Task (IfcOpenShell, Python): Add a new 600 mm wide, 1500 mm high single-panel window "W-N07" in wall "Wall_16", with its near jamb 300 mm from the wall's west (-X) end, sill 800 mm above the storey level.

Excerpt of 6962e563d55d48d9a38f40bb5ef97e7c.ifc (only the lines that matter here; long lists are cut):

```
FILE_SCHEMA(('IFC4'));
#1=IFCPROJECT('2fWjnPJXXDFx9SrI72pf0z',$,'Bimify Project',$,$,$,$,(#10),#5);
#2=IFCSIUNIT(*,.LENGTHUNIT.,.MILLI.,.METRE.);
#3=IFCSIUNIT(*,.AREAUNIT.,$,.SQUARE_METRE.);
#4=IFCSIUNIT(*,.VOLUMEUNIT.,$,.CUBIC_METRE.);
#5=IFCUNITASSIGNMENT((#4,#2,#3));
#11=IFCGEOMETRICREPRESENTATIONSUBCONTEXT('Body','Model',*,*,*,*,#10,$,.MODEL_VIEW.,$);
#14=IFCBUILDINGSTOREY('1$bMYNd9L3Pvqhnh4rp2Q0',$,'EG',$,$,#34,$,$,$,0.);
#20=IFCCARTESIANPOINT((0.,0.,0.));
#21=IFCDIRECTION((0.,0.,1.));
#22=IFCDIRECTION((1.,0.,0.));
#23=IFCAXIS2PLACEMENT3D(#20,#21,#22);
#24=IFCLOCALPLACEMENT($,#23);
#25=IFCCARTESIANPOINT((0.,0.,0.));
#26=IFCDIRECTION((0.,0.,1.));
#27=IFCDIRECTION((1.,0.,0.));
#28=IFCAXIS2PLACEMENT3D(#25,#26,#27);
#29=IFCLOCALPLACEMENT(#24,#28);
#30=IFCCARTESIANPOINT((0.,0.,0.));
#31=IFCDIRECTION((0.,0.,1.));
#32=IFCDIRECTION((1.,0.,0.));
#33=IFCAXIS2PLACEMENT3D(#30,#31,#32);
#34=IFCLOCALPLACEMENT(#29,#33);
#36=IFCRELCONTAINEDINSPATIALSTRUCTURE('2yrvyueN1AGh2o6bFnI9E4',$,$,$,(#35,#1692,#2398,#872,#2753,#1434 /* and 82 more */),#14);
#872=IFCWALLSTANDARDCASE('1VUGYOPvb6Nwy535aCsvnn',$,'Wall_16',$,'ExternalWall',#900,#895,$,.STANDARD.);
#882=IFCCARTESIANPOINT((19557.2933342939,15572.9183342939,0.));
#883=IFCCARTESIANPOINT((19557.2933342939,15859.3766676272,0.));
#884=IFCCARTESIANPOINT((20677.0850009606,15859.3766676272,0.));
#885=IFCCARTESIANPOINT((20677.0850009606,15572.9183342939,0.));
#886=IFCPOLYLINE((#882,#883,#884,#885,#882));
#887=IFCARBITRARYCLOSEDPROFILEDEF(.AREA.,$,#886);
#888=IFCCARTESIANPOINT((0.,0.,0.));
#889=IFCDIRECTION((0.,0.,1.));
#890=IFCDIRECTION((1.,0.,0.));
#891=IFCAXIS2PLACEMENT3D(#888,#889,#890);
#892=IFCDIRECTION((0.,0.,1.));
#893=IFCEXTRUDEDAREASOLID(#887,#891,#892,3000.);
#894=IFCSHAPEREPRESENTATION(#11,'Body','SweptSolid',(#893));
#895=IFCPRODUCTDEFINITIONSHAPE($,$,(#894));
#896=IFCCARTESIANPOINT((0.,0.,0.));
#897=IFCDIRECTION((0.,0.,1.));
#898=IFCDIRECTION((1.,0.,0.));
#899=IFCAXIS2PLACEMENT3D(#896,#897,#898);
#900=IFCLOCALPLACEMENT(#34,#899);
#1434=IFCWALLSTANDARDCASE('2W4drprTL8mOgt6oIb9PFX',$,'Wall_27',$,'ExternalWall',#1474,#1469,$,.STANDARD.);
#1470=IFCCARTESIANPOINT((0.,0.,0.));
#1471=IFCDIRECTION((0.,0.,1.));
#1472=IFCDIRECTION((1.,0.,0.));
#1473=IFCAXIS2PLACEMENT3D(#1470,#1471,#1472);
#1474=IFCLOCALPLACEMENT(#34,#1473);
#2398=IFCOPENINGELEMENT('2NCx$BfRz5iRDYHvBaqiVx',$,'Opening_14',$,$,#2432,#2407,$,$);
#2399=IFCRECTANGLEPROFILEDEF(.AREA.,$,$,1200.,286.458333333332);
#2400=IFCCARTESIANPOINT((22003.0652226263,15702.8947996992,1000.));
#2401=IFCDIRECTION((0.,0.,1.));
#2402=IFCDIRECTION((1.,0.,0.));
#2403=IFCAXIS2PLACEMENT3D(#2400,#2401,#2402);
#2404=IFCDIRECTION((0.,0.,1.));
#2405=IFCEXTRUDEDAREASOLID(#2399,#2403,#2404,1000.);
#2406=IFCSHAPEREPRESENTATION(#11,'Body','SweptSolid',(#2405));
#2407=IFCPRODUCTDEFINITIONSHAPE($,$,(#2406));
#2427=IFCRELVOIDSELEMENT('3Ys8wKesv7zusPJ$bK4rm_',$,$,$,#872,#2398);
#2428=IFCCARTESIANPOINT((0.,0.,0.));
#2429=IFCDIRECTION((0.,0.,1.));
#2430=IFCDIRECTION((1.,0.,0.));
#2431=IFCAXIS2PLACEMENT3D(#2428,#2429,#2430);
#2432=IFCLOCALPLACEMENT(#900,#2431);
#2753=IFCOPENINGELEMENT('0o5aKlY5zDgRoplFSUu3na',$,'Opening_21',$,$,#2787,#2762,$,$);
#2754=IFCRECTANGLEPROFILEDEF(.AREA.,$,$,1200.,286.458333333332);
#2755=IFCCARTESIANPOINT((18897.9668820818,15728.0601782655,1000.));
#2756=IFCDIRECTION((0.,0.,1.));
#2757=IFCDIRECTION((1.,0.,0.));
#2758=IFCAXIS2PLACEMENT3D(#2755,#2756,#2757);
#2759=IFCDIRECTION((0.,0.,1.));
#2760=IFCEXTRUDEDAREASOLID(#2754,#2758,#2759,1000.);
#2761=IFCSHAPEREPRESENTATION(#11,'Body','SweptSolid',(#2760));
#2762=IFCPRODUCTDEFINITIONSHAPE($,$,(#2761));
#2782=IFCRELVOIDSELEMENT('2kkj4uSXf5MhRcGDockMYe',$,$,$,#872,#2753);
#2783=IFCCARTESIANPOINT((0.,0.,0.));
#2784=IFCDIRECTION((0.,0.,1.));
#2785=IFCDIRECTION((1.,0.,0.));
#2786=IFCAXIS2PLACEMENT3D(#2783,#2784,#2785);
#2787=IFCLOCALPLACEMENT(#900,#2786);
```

```python
import numpy as np
import ifcopenshell
import ifcopenshell.api.feature
import ifcopenshell.api.geometry
import ifcopenshell.api.root
import ifcopenshell.api.spatial
import ifcopenshell.geom
import ifcopenshell.util.element
import ifcopenshell.util.placement
import ifcopenshell.util.representation
import ifcopenshell.util.shape
import ifcopenshell.util.unit

model = ifcopenshell.open("6962e563d55d48d9a38f40bb5ef97e7c.ifc")
unit_scale = ifcopenshell.util.unit.calculate_unit_scale(model)
settings = ifcopenshell.geom.settings()


def volume(element):
    """Net volume in cubic metres, openings subtracted."""
    shape = ifcopenshell.geom.create_shape(settings, element)
    return ifcopenshell.util.shape.get_volume(shape.geometry)


wall = model.by_guid("1VUGYOPvb6Nwy535aCsvnn")
storey = ifcopenshell.util.element.get_container(wall, ifc_class="IfcBuildingStorey")
context = ifcopenshell.util.representation.get_context(model, "Model", "Body", "MODEL_VIEW")
before = volume(wall)

width, height, from_end, sill = 0.6, 1.5, 0.3, 0.8  # metres

# The wall runs along its own X axis, and the end named is its -X end.
wall_shape = ifcopenshell.geom.create_shape(settings, wall)
x, y, z = ifcopenshell.util.shape.get_vertices(wall_shape.geometry).T
start = x.min() + from_end
face, thickness = float(y.min()), float(y.max() - y.min())
wall_matrix = ifcopenshell.util.placement.get_local_placement(wall.ObjectPlacement)
level = ifcopenshell.util.placement.get_local_placement(storey.ObjectPlacement)[2, 3]


def in_wall(x, y):
    """Placement at x, y metres in the wall's axes, at sill height."""
    matrix = wall_matrix.copy()
    matrix[:, 3] = wall_matrix @ np.array([x / unit_scale, y / unit_scale, 0.0, 1.0])
    matrix[2, 3] = level + sill / unit_scale
    return matrix


# Opening: a box that overshoots both wall faces by 50 mm.
opening = ifcopenshell.api.root.create_entity(model, ifc_class="IfcOpeningElement", predefined_type="OPENING")
box = ifcopenshell.api.geometry.add_wall_representation(
    model, context=context, length=width, height=height, thickness=thickness + 0.1
)
ifcopenshell.api.geometry.assign_representation(model, product=opening, representation=box)
ifcopenshell.api.geometry.edit_object_placement(model, product=opening, matrix=in_wall(start, face - 0.05), is_si=False)
ifcopenshell.api.feature.add_feature(model, feature=opening, element=wall)

window = ifcopenshell.api.root.create_entity(model, ifc_class="IfcWindow", name="W-N07", predefined_type="WINDOW")
window.OverallWidth, window.OverallHeight = width / unit_scale, height / unit_scale
window.PartitioningType = "SINGLE_PANEL"
body = ifcopenshell.api.geometry.add_window_representation(
    model,
    context=context,
    overall_width=window.OverallWidth,
    overall_height=window.OverallHeight,
    partition_type="SINGLE_PANEL",
)
ifcopenshell.api.geometry.assign_representation(model, product=window, representation=body)
ifcopenshell.api.spatial.assign_container(model, products=[window], relating_structure=storey)
ifcopenshell.api.feature.add_filling(model, opening=opening, element=window)

# Centre the window in the wall's thickness.
ifcopenshell.api.geometry.edit_object_placement(model, product=window, matrix=in_wall(start, face), is_si=False)
window_shape = ifcopenshell.geom.create_shape(settings, window)
depth = ifcopenshell.util.shape.get_vertices(window_shape.geometry)[:, 1]
offset = face + thickness / 2 - (depth.min() + depth.max()) / 2
ifcopenshell.api.geometry.edit_object_placement(model, product=window, matrix=in_wall(start, offset), is_si=False)

after = volume(wall)

print(f"wall volume {before:.3f} -> {after:.3f} m3")

model.write("6962e563d55d48d9a38f40bb5ef97e7c_v2.ifc")
```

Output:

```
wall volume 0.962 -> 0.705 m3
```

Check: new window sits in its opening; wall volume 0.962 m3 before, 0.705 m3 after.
